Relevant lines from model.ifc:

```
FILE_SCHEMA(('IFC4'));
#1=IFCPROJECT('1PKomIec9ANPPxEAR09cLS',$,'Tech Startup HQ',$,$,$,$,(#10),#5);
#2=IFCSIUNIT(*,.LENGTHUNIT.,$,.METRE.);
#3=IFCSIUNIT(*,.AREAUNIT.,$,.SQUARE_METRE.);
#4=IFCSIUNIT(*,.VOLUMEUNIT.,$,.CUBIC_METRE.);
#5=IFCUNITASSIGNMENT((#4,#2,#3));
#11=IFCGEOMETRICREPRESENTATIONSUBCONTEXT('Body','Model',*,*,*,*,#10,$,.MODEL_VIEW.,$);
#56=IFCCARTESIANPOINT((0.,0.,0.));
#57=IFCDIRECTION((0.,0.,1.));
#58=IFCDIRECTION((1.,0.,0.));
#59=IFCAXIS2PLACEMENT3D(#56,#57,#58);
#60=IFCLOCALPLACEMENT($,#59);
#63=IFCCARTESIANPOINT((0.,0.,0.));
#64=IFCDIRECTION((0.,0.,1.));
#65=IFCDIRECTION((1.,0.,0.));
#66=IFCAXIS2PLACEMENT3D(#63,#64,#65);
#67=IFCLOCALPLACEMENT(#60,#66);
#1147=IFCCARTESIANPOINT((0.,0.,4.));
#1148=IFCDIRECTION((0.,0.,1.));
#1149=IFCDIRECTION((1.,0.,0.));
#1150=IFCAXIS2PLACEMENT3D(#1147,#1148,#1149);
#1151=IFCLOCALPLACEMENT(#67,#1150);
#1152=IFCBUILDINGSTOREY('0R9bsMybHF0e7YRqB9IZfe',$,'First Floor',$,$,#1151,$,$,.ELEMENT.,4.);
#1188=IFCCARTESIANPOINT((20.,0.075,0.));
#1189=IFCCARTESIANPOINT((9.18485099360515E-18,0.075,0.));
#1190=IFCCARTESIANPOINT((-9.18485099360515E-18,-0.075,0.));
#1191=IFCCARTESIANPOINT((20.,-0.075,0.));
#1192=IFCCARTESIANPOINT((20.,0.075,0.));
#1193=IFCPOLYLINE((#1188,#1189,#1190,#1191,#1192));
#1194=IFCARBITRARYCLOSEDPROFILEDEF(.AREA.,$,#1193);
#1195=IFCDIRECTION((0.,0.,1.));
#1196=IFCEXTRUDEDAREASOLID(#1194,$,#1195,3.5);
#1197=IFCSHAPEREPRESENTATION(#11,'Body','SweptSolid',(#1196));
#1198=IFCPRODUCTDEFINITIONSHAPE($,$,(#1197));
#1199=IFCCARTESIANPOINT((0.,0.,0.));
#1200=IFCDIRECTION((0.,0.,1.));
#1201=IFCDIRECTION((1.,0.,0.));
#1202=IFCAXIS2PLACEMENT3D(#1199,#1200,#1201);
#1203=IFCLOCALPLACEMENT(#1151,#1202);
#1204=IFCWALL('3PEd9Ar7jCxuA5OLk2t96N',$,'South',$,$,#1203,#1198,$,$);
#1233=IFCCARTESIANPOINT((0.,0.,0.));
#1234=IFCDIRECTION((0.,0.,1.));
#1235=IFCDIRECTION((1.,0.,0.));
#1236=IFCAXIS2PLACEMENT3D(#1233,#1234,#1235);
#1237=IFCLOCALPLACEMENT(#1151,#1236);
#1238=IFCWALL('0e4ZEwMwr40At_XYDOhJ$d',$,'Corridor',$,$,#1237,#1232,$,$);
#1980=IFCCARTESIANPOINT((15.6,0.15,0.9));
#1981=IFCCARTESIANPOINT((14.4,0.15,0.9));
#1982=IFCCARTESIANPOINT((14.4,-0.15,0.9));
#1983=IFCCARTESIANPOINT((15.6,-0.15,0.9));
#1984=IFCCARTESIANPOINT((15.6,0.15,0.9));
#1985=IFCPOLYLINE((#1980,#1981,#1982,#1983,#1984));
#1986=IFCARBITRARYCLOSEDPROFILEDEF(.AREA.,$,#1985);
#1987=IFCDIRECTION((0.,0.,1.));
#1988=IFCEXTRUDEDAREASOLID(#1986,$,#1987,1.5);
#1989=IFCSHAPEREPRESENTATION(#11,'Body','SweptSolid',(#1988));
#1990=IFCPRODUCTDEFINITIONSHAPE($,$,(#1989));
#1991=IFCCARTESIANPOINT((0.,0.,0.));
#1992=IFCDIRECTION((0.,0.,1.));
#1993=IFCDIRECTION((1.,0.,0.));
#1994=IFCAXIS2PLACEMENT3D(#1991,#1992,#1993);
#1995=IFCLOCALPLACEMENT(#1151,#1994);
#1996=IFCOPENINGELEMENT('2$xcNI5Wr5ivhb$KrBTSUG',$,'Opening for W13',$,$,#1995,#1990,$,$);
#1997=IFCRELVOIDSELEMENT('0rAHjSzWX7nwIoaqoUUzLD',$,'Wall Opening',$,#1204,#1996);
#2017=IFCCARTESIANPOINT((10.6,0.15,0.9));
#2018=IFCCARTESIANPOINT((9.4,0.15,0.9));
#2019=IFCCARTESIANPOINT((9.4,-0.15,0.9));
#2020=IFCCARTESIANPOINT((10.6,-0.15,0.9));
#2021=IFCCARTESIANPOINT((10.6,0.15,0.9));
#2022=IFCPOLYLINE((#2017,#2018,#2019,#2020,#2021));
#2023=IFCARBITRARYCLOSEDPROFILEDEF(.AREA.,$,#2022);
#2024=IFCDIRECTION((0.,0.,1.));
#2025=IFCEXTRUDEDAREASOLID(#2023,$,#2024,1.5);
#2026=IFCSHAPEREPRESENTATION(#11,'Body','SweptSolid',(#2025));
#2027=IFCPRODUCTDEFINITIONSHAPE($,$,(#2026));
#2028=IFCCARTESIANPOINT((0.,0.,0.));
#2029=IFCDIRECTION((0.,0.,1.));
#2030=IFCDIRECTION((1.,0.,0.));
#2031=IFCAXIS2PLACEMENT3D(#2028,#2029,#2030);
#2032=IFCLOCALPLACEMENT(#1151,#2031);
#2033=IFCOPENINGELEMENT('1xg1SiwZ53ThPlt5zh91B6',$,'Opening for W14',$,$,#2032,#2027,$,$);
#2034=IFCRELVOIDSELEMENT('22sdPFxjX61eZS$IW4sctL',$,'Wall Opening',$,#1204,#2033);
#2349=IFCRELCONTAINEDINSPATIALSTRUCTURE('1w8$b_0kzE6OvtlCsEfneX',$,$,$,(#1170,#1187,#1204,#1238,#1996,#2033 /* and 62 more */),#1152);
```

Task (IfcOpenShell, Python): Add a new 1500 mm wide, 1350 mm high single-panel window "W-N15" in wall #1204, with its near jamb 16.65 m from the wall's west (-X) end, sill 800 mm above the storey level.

```python
import numpy as np
import ifcopenshell
import ifcopenshell.api.feature
import ifcopenshell.api.geometry
import ifcopenshell.api.root
import ifcopenshell.api.spatial
import ifcopenshell.geom
import ifcopenshell.util.element
import ifcopenshell.util.placement
import ifcopenshell.util.representation
import ifcopenshell.util.shape
import ifcopenshell.util.unit

model = ifcopenshell.open("model.ifc")
unit_scale = ifcopenshell.util.unit.calculate_unit_scale(model)
settings = ifcopenshell.geom.settings()


def volume(element):
    """Net volume in cubic metres, openings subtracted."""
    shape = ifcopenshell.geom.create_shape(settings, element)
    return ifcopenshell.util.shape.get_volume(shape.geometry)


wall = model.by_guid("3PEd9Ar7jCxuA5OLk2t96N")
storey = ifcopenshell.util.element.get_container(wall, ifc_class="IfcBuildingStorey")
context = ifcopenshell.util.representation.get_context(model, "Model", "Body", "MODEL_VIEW")
before = volume(wall)

width, height, from_end, sill = 1.5, 1.35, 16.65, 0.8  # metres

# The wall runs along its own X axis, and the end named is its -X end.
wall_shape = ifcopenshell.geom.create_shape(settings, wall)
x, y, z = ifcopenshell.util.shape.get_vertices(wall_shape.geometry).T
start = x.min() + from_end
face, thickness = float(y.min()), float(y.max() - y.min())
wall_matrix = ifcopenshell.util.placement.get_local_placement(wall.ObjectPlacement)
level = ifcopenshell.util.placement.get_local_placement(storey.ObjectPlacement)[2, 3]


def in_wall(x, y):
    """Placement at x, y metres in the wall's axes, at sill height."""
    matrix = wall_matrix.copy()
    matrix[:, 3] = wall_matrix @ np.array([x / unit_scale, y / unit_scale, 0.0, 1.0])
    matrix[2, 3] = level + sill / unit_scale
    return matrix


# Opening: a box that overshoots both wall faces by 50 mm.
opening = ifcopenshell.api.root.create_entity(model, ifc_class="IfcOpeningElement", predefined_type="OPENING")
box = ifcopenshell.api.geometry.add_wall_representation(
    model, context=context, length=width, height=height, thickness=thickness + 0.1
)
ifcopenshell.api.geometry.assign_representation(model, product=opening, representation=box)
ifcopenshell.api.geometry.edit_object_placement(model, product=opening, matrix=in_wall(start, face - 0.05), is_si=False)
ifcopenshell.api.feature.add_feature(model, feature=opening, element=wall)

window = ifcopenshell.api.root.create_entity(model, ifc_class="IfcWindow", name="W-N15", predefined_type="WINDOW")
window.OverallWidth, window.OverallHeight = width / unit_scale, height / unit_scale
window.PartitioningType = "SINGLE_PANEL"
body = ifcopenshell.api.geometry.add_window_representation(
    model,
    context=context,
    overall_width=window.OverallWidth,
    overall_height=window.OverallHeight,
    partition_type="SINGLE_PANEL",
)
ifcopenshell.api.geometry.assign_representation(model, product=window, representation=body)
ifcopenshell.api.spatial.assign_container(model, products=[window], relating_structure=storey)
ifcopenshell.api.feature.add_filling(model, opening=opening, element=window)

# Centre the window in the wall's thickness.
ifcopenshell.api.geometry.edit_object_placement(model, product=window, matrix=in_wall(start, face), is_si=False)
window_shape = ifcopenshell.geom.create_shape(settings, window)
depth = ifcopenshell.util.shape.get_vertices(window_shape.geometry)[:, 1]
offset = face + thickness / 2 - (depth.min() + depth.max()) / 2
ifcopenshell.api.geometry.edit_object_placement(model, product=window, matrix=in_wall(start, offset), is_si=False)

after = volume(wall)

print(f"wall volume {before:.3f} -> {after:.3f} m3")

model.write("model_v2.ifc")
```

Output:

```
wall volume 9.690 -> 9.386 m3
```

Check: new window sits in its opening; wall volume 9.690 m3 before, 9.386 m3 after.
